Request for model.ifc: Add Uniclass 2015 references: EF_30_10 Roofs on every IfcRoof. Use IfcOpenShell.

First a look at what the model holds.

```python
import ifcopenshell

model = ifcopenshell.open("model.ifc")
print(model.schema)
print("classifications:", [c.Name for c in model.by_type("IfcClassification")])
for ifc_class in ("IfcDoor", "IfcRoof", "IfcStair", "IfcWall", "IfcWindow"):
    print(ifc_class, len(model.by_type(ifc_class)))
```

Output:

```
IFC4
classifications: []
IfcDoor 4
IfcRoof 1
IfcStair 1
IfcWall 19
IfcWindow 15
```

```python
import ifcopenshell
import ifcopenshell.api.classification

model = ifcopenshell.open("model.ifc")

system = ifcopenshell.api.classification.add_classification(model, classification="Uniclass 2015")

codes = {
    "IfcRoof": ("EF_30_10", "Roofs"),
}
for ifc_class, (code, name) in codes.items():
    products = model.by_type(ifc_class)
    ifcopenshell.api.classification.add_reference(
        model, products=products, classification=system, identification=code, name=name
    )
    print(code, len(products))

model.write("model_updated.ifc")
```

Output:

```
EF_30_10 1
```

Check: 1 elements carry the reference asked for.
